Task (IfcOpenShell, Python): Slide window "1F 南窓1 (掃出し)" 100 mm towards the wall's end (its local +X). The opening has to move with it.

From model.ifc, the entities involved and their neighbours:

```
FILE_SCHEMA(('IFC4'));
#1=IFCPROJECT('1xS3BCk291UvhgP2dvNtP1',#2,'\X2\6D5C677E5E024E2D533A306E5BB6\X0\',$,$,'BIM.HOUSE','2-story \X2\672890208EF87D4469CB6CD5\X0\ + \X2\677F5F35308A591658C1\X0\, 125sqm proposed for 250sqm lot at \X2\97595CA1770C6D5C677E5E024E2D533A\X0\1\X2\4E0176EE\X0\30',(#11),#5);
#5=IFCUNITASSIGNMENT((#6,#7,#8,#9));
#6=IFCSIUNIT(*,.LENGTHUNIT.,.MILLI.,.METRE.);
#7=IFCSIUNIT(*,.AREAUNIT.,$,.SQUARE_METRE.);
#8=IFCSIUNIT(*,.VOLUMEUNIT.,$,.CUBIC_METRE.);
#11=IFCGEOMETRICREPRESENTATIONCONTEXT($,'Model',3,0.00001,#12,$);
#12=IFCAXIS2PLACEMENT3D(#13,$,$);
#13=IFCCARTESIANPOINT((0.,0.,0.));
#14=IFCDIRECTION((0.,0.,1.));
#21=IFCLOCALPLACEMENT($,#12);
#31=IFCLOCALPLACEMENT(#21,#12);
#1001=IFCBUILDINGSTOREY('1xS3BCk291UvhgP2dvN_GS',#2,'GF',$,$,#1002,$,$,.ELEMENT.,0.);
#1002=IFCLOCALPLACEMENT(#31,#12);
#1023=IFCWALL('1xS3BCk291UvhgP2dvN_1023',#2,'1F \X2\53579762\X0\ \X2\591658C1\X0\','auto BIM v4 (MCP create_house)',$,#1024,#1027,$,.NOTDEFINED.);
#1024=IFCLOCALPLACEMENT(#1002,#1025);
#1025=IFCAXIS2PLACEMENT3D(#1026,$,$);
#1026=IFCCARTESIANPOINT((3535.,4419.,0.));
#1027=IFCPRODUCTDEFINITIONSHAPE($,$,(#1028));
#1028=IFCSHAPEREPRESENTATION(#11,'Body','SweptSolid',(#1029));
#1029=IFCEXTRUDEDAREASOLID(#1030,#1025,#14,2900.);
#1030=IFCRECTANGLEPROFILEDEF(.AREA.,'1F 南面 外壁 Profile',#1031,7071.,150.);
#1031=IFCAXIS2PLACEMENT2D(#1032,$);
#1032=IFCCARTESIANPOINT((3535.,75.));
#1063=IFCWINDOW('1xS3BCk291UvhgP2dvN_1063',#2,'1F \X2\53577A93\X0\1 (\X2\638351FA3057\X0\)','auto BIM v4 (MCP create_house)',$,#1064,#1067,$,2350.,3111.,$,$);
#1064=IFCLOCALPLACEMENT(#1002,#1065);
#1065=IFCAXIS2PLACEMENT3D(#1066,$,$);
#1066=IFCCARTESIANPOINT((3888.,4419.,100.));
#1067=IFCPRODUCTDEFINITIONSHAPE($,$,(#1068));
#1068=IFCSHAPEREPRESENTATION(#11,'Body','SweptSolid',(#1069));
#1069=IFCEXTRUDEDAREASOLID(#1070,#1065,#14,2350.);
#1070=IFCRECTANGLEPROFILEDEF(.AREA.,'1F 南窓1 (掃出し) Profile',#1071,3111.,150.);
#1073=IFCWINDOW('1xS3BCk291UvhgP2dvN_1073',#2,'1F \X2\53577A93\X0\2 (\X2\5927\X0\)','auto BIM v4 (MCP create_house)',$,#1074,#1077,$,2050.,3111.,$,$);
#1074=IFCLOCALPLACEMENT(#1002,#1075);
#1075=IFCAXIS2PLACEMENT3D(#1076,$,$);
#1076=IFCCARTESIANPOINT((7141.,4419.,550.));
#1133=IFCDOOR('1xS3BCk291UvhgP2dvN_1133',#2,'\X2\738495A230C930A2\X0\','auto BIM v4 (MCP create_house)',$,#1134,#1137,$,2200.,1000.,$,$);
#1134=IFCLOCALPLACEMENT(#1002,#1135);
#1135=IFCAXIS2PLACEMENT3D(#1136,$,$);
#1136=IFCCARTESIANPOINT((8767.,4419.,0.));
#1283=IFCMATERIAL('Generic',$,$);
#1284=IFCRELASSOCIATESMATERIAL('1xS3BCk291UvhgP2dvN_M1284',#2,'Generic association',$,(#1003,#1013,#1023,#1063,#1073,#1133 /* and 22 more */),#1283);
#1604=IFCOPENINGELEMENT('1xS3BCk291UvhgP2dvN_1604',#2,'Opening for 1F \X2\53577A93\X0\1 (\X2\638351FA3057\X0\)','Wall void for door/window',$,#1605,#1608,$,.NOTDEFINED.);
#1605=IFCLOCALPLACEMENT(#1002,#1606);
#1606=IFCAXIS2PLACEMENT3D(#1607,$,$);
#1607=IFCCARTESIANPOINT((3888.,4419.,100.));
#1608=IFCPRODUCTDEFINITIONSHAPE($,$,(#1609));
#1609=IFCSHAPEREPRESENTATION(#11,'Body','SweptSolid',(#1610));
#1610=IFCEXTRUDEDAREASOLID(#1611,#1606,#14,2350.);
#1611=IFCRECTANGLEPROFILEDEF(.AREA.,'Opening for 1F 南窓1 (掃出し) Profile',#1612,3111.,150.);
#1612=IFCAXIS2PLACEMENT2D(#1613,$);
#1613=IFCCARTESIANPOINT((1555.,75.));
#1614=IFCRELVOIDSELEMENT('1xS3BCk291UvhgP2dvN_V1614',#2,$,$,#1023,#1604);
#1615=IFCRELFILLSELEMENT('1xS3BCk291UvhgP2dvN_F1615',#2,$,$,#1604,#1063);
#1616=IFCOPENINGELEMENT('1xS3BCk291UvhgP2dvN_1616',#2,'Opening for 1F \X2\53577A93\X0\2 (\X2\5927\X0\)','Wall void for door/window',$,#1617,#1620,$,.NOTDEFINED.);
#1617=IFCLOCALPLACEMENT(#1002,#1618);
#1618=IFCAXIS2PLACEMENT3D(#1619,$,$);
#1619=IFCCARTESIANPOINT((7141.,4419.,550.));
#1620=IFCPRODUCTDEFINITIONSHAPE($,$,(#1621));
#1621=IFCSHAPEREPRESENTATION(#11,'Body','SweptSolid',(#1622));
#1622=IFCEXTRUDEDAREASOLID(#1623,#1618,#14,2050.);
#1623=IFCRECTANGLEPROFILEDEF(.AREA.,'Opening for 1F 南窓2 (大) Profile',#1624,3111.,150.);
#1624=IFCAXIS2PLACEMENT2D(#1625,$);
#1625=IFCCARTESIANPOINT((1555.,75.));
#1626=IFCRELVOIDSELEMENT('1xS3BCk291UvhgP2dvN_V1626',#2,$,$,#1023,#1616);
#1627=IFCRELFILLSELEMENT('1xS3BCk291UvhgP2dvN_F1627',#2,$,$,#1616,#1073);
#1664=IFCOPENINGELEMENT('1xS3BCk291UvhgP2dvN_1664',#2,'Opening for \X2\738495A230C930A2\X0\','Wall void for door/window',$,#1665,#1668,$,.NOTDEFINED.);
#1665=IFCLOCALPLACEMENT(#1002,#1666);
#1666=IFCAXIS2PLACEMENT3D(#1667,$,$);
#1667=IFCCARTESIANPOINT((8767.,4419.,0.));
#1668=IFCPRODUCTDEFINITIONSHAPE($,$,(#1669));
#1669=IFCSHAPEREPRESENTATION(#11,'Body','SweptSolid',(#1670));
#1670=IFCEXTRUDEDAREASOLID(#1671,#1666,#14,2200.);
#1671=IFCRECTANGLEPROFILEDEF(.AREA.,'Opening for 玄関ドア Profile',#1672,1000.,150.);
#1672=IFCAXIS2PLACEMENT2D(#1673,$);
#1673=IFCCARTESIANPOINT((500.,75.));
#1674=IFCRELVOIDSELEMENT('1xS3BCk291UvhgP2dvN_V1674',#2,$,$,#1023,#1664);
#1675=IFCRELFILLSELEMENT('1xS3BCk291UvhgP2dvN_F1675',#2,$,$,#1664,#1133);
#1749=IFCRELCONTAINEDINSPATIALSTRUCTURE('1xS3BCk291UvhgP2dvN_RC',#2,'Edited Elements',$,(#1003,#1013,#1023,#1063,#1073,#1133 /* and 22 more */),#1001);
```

```python
import ifcopenshell
import ifcopenshell.api.geometry
import ifcopenshell.util.placement

model = ifcopenshell.open("model.ifc")

window = model.by_guid("1xS3BCk291UvhgP2dvN_1063")
opening = window.FillsVoids[0].RelatingOpeningElement
wall = opening.VoidsElements[0].RelatingBuildingElement

wall_matrix = ifcopenshell.util.placement.get_local_placement(wall.ObjectPlacement)
shift = wall_matrix[:3, 0] * 100.0
before = ifcopenshell.util.placement.get_local_placement(window.ObjectPlacement)[:3, 3].copy()

# The window is not placed relative to its opening, so move both.
for product in (opening, window):
    matrix = ifcopenshell.util.placement.get_local_placement(product.ObjectPlacement)
    matrix[:3, 3] += shift
    ifcopenshell.api.geometry.edit_object_placement(model, product=product, matrix=matrix, is_si=False)

after = ifcopenshell.util.placement.get_local_placement(window.ObjectPlacement)[:3, 3]
print("window moved by", (after - before).round(3) + 0.0)

model.write("model_edited.ifc")
```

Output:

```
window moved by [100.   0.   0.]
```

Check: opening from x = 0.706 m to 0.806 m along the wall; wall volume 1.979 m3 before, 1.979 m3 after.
